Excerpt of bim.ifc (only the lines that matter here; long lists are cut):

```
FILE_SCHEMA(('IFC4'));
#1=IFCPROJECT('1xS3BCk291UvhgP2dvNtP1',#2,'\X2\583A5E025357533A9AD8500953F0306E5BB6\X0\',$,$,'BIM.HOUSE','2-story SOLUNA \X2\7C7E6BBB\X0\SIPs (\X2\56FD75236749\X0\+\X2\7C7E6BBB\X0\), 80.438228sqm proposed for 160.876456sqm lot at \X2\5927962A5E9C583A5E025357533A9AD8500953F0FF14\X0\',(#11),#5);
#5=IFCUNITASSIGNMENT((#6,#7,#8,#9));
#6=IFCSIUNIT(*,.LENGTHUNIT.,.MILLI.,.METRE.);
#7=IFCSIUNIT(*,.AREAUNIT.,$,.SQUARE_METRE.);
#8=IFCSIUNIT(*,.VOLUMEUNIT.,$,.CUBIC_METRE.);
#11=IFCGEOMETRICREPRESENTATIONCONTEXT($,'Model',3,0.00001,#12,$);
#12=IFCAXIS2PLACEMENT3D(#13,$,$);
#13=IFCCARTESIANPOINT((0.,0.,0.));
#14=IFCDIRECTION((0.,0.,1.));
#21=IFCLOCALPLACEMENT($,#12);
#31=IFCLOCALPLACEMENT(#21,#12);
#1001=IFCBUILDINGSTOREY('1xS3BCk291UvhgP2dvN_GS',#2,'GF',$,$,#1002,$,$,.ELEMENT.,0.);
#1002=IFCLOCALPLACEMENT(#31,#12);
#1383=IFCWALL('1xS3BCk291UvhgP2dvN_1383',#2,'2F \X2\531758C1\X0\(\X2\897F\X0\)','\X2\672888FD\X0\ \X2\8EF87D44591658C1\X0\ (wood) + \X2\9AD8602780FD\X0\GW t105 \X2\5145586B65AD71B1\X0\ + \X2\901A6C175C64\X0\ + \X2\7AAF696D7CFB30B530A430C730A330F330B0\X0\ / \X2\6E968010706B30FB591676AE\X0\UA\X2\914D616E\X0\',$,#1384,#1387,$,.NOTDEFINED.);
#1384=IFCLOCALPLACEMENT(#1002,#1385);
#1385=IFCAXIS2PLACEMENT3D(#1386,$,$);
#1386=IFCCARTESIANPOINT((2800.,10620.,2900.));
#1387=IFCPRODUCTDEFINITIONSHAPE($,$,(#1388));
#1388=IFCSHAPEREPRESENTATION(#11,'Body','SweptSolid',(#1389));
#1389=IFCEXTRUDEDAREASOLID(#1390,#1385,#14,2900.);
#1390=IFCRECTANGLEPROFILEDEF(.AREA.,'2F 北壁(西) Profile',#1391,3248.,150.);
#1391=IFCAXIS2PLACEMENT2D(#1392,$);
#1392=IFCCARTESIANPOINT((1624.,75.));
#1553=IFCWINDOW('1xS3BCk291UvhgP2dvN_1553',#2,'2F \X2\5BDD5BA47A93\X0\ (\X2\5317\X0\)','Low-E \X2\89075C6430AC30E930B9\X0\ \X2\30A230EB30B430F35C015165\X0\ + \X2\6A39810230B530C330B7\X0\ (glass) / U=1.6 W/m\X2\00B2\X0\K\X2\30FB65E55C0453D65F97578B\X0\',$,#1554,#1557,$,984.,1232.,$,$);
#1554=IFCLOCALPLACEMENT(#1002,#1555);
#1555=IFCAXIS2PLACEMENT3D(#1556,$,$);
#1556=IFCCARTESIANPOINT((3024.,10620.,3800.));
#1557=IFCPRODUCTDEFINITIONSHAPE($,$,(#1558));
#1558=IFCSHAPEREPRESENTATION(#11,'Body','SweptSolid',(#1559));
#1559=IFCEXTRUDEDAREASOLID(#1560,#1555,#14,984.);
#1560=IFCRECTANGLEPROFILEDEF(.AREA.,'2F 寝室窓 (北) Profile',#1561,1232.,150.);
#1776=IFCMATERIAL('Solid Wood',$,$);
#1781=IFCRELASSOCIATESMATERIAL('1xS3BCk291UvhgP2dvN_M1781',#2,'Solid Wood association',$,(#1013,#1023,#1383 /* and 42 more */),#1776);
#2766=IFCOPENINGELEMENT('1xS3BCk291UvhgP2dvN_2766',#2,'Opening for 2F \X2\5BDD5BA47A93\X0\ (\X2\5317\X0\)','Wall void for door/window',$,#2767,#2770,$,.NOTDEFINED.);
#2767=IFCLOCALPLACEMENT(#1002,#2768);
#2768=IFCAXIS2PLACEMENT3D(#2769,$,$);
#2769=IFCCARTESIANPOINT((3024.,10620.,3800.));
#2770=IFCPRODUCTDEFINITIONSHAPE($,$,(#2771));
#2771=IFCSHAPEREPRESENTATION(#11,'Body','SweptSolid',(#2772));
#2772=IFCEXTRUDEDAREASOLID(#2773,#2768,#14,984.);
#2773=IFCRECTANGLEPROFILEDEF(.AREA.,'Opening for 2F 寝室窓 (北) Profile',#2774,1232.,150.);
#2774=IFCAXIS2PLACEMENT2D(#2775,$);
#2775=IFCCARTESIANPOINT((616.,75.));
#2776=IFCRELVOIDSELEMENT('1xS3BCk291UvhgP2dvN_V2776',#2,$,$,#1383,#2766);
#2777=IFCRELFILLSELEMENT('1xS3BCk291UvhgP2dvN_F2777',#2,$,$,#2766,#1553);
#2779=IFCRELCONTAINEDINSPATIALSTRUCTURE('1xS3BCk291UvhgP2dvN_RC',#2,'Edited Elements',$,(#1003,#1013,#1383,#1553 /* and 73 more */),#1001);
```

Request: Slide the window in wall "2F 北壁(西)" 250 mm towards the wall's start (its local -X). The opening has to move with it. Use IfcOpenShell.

```python
import ifcopenshell
import ifcopenshell.api.geometry
import ifcopenshell.util.placement
import ifcopenshell.util.unit

model = ifcopenshell.open("bim.ifc")
unit_scale = ifcopenshell.util.unit.calculate_unit_scale(model)

window = model.by_id(1553)
opening = window.FillsVoids[0].RelatingOpeningElement
wall = opening.VoidsElements[0].RelatingBuildingElement

wall_matrix = ifcopenshell.util.placement.get_local_placement(wall.ObjectPlacement)
shift = wall_matrix[:3, 0] * -0.25 / unit_scale
before = ifcopenshell.util.placement.get_local_placement(window.ObjectPlacement)[:3, 3].copy()

# The window is not placed relative to its opening, so move both.
for product in (opening, window):
    matrix = ifcopenshell.util.placement.get_local_placement(product.ObjectPlacement)
    matrix[:3, 3] += shift
    ifcopenshell.api.geometry.edit_object_placement(model, product=product, matrix=matrix, is_si=False)

after = ifcopenshell.util.placement.get_local_placement(window.ObjectPlacement)[:3, 3]
print("window moved by", (after - before).round(3) + 0.0)

model.write("bim_updated.ifc")
```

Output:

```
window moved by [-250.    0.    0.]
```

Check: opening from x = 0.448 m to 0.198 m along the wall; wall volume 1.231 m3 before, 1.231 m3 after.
